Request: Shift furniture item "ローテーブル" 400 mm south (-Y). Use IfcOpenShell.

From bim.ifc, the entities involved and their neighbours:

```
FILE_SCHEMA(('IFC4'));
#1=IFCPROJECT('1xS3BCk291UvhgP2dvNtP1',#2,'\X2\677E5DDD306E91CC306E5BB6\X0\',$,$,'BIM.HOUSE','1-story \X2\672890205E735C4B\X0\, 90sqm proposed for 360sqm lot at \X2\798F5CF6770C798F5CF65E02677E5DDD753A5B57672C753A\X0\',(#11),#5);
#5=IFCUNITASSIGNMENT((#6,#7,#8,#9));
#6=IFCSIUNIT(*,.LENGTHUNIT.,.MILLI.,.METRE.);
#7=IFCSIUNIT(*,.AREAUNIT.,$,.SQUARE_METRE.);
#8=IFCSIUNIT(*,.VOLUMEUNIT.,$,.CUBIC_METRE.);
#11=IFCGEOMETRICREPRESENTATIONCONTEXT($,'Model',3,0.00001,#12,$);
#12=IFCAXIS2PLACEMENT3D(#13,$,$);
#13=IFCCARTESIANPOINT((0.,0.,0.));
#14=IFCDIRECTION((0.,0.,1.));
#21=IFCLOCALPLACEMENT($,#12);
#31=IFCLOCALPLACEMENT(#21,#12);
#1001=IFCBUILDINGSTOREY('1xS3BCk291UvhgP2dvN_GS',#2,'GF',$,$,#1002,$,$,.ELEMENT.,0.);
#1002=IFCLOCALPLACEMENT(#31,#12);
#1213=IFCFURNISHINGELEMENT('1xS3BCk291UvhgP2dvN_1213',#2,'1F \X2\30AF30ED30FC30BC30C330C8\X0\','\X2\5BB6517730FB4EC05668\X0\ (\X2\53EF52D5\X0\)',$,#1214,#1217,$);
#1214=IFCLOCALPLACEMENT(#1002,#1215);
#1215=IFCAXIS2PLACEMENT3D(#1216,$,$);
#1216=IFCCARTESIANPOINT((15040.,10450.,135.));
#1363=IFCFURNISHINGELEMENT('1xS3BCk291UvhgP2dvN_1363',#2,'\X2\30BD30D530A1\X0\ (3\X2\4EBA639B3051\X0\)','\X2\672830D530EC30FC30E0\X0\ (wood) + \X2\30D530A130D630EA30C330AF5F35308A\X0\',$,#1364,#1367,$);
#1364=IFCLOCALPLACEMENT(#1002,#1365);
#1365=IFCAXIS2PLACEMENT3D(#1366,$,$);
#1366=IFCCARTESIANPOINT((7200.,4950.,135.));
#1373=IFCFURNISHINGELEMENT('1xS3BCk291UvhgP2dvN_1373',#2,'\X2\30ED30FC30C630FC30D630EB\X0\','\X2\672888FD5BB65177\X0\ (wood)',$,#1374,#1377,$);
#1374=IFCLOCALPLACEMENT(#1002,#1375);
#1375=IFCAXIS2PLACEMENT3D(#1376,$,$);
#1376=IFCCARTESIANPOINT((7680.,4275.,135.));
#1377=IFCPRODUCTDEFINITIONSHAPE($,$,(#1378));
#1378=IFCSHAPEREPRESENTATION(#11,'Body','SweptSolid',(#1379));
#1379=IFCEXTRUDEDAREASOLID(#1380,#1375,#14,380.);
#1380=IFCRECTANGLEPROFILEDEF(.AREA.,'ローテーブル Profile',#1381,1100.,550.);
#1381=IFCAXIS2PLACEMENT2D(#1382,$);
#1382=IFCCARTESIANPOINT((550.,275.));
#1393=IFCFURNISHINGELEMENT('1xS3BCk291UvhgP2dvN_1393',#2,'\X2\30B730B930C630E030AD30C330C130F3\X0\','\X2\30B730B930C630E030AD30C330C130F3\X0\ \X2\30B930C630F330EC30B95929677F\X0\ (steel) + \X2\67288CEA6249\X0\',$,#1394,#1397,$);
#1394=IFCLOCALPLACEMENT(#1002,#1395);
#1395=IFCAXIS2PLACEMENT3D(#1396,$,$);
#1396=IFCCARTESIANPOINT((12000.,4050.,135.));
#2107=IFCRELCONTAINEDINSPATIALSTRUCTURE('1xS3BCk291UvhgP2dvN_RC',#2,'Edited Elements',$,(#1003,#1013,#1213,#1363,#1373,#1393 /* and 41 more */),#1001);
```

```python
import ifcopenshell
import ifcopenshell.api.geometry
import ifcopenshell.util.placement
import ifcopenshell.util.unit

model = ifcopenshell.open("bim.ifc")
unit_scale = ifcopenshell.util.unit.calculate_unit_scale(model)

item = model.by_guid("1xS3BCk291UvhgP2dvN_1373")
matrix = ifcopenshell.util.placement.get_local_placement(item.ObjectPlacement)
matrix[1, 3] -= 0.4 / unit_scale
ifcopenshell.api.geometry.edit_object_placement(model, product=item, matrix=matrix, is_si=False)

print(ifcopenshell.util.placement.get_local_placement(item.ObjectPlacement).round(3) + 0.0)

model.write("bim_edited.ifc")
```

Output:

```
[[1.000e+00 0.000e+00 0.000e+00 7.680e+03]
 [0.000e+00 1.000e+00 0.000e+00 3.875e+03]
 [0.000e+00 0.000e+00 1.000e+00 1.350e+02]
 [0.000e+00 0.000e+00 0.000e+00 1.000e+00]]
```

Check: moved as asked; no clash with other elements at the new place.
